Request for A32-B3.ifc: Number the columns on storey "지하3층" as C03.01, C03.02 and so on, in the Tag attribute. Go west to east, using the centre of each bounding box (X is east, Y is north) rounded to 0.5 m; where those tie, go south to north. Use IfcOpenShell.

First a look at what the model holds.

```python
import ifcopenshell
import ifcopenshell.util.element
import ifcopenshell.util.placement

model = ifcopenshell.open("A32-B3.ifc")
print(model.schema)
storey = next(s for s in model.by_type("IfcBuildingStorey") if s.Name == "지하3층")
columns = [e for e in ifcopenshell.util.element.get_decomposition(storey) if e.is_a("IfcColumn")]
for e in sorted(columns, key=lambda e: e.id()):
    origin = ifcopenshell.util.placement.get_local_placement(e.ObjectPlacement)[:3, 3]
    print(e.id(), e.Tag, e.Name, origin.round(2) + 0.0, sep=" | ")
```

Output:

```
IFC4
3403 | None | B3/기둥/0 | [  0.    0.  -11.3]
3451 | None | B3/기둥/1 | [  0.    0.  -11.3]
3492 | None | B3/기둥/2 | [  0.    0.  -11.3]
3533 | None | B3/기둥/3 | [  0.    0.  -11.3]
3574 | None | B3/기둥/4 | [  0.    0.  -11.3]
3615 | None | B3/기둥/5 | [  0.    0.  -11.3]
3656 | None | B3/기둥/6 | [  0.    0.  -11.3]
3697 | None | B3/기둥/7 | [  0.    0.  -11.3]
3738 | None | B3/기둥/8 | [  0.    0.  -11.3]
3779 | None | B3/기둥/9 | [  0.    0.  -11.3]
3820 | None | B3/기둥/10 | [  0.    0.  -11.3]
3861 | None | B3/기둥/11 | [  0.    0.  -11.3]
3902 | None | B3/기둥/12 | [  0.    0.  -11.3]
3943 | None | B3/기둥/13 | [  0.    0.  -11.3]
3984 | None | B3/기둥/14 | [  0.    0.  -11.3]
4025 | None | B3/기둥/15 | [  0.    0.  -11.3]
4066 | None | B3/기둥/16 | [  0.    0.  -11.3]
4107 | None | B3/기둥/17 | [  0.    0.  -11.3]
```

```python
import ifcopenshell
import ifcopenshell.geom
import ifcopenshell.util.element
import ifcopenshell.util.shape

model = ifcopenshell.open("A32-B3.ifc")
settings = ifcopenshell.geom.settings()
settings.set("use-world-coords", True)


def centre(element):
    shape = ifcopenshell.geom.create_shape(settings, element)
    return ifcopenshell.util.shape.get_bbox_centroid(shape.geometry)


storey = next(s for s in model.by_type("IfcBuildingStorey") if s.Name == "지하3층")
columns = [e for e in ifcopenshell.util.element.get_decomposition(storey) if e.is_a("IfcColumn")]

# Insertion points can sit at a corner or the storey origin, so sort by the geometry (in metres).
centres = {e: centre(e) for e in columns}
columns.sort(key=lambda e: (round(centres[e][0] / 0.5), centres[e][1]))

for i, e in enumerate(columns, start=1):
    number = f"C03.{i:02d}"
    e.Tag = number
    print(e.id(), number)

model.write("A32-B3-out.ifc")
```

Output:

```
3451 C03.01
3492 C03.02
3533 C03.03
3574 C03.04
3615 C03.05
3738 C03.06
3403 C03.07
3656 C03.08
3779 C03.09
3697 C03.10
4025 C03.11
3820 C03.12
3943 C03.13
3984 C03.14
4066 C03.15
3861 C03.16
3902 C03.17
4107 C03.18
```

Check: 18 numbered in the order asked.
